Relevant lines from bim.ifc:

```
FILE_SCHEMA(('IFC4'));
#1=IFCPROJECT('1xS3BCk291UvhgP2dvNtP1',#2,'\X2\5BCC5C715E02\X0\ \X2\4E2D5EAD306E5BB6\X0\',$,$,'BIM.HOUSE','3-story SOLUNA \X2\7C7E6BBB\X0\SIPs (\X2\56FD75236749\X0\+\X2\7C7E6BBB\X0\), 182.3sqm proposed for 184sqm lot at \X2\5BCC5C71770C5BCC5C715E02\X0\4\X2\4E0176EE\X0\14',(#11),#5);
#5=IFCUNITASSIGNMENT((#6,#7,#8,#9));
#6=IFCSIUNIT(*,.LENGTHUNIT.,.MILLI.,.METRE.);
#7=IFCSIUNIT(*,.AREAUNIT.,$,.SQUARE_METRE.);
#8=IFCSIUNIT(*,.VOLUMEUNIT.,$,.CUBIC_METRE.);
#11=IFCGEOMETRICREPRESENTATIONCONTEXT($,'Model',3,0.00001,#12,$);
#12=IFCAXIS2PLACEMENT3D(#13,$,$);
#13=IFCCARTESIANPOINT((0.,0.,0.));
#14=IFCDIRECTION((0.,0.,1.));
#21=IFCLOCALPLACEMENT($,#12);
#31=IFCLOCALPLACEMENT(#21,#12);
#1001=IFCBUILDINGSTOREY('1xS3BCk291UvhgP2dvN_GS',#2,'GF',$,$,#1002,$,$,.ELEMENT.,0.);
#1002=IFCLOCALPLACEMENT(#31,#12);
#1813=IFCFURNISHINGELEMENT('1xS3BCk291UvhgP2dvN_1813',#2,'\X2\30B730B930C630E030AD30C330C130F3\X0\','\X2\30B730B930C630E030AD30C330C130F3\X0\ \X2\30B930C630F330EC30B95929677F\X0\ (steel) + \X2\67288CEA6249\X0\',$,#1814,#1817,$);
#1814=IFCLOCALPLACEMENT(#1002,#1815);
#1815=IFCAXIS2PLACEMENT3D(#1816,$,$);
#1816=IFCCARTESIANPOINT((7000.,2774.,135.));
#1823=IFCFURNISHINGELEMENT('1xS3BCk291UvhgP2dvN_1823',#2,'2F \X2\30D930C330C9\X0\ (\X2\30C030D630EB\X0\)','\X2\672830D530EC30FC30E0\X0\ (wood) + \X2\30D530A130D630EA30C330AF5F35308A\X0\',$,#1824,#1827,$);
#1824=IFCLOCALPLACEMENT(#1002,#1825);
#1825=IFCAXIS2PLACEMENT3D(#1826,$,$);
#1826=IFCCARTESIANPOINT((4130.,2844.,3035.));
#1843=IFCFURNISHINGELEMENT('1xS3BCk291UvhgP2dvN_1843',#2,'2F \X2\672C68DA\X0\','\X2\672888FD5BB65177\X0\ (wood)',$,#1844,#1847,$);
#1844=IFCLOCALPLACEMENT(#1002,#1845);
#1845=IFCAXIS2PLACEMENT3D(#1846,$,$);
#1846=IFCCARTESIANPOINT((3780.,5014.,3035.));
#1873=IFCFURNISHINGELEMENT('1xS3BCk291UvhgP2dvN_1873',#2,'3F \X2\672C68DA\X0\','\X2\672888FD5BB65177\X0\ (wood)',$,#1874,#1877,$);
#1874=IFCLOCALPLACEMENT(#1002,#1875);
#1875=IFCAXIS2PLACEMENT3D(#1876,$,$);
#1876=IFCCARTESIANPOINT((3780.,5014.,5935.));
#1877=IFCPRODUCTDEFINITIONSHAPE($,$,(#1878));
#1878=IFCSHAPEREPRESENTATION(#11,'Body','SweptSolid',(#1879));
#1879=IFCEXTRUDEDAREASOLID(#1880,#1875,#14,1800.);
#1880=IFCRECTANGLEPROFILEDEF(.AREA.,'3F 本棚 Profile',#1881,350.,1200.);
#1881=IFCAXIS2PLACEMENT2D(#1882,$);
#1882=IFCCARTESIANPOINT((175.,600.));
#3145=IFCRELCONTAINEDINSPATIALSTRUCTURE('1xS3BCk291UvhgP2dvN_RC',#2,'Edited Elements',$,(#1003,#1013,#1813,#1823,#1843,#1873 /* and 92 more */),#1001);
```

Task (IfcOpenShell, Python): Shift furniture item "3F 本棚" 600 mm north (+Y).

```python
import ifcopenshell
import ifcopenshell.api.geometry
import ifcopenshell.util.placement
import ifcopenshell.util.unit

model = ifcopenshell.open("bim.ifc")
unit_scale = ifcopenshell.util.unit.calculate_unit_scale(model)

item = model.by_guid("1xS3BCk291UvhgP2dvN_1873")
matrix = ifcopenshell.util.placement.get_local_placement(item.ObjectPlacement)
matrix[1, 3] += 0.6 / unit_scale
ifcopenshell.api.geometry.edit_object_placement(model, product=item, matrix=matrix, is_si=False)

print(ifcopenshell.util.placement.get_local_placement(item.ObjectPlacement).round(3) + 0.0)

model.write("bim_edited.ifc")
```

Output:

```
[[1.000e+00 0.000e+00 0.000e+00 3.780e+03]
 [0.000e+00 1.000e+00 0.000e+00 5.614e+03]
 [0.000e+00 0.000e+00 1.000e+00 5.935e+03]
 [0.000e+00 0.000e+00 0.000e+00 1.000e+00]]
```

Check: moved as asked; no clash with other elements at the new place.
